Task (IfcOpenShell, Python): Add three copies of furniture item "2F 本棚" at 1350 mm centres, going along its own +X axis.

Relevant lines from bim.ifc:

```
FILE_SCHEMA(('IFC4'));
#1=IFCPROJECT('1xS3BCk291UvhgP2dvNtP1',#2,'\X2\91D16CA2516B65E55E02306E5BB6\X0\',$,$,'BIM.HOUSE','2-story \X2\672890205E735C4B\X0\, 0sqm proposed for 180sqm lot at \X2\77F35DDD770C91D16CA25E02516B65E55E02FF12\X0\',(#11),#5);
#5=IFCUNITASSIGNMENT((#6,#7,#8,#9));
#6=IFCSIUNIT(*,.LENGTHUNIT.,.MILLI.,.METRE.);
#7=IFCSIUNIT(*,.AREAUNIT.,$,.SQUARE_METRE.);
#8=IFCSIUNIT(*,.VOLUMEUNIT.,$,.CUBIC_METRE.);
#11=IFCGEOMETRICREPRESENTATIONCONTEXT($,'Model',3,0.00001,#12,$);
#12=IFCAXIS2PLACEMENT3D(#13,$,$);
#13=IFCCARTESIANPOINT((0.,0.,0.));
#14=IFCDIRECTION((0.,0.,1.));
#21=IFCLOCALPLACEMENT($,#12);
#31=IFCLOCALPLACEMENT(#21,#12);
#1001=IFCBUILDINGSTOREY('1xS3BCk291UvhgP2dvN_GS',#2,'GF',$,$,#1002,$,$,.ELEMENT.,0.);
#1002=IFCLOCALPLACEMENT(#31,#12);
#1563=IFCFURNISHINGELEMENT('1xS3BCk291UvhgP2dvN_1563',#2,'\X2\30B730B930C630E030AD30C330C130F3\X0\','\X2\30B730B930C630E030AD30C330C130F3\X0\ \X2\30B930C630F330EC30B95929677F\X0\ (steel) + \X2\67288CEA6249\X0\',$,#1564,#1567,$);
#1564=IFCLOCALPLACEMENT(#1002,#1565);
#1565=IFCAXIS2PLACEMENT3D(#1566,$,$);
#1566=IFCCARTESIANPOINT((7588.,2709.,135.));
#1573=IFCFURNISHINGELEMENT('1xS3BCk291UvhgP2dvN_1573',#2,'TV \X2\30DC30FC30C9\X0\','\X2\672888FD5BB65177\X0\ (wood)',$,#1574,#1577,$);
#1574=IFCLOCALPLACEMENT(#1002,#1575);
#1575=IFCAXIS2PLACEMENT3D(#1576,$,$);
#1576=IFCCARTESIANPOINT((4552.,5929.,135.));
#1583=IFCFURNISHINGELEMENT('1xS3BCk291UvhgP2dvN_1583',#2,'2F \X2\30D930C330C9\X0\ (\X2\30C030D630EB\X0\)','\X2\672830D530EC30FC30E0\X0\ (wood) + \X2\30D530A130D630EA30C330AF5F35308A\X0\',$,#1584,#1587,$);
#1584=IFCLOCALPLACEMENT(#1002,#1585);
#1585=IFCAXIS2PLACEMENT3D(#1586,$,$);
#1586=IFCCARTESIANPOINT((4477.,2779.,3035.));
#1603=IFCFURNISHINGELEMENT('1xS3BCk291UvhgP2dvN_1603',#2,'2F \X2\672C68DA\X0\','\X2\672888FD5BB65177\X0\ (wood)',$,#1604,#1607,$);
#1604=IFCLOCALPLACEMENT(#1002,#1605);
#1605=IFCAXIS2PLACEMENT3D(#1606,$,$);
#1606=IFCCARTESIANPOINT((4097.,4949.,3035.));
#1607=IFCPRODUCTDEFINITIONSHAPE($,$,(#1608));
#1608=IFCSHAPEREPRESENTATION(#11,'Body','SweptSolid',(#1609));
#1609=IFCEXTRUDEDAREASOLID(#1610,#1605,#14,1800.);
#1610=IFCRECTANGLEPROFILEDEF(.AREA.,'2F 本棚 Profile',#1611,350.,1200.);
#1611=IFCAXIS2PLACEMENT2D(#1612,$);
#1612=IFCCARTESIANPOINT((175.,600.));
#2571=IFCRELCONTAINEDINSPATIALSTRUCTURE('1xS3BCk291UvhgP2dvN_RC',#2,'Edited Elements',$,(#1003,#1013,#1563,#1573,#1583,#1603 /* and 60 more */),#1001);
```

```python
import ifcopenshell
import ifcopenshell.api.geometry
import ifcopenshell.api.root
import ifcopenshell.util.element
import ifcopenshell.util.placement

model = ifcopenshell.open("bim.ifc")


def reuse_history(source, copy):
    """copy_class also copies each property set's owner history, people and application; keep the originals."""
    for rel in copy.IsDefinedBy:
        if rel.is_a("IfcRelDefinesByProperties") and (history := rel.RelatingPropertyDefinition.OwnerHistory):
            rel.RelatingPropertyDefinition.OwnerHistory = source.OwnerHistory
            ifcopenshell.util.element.remove_deep2(model, history)


source = model.by_guid("1xS3BCk291UvhgP2dvN_1603")
base = ifcopenshell.util.placement.get_local_placement(source.ObjectPlacement)
step = base[:3, 0] * 1350.0

for i in range(1, 4):
    copy = ifcopenshell.api.root.copy_class(model, product=source)
    copy.Representation = ifcopenshell.util.element.copy_deep(
        model, source.Representation, exclude=["IfcGeometricRepresentationContext", "IfcRepresentationMap"]
    )
    reuse_history(source, copy)
    matrix = base.copy()
    matrix[:3, 3] += i * step
    print("added at", matrix[:3, 3].round(3) + 0.0)
    ifcopenshell.api.geometry.edit_object_placement(model, product=copy, matrix=matrix, is_si=False)

model.write("bim-out.ifc")
```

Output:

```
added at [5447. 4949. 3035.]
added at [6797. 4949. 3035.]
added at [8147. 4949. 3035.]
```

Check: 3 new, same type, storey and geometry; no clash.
